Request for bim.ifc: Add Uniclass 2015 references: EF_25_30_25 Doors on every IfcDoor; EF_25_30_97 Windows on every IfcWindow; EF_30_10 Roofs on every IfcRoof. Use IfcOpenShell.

First a look at what the model holds.

```python
import ifcopenshell

model = ifcopenshell.open("bim.ifc")
print(model.schema)
print("classifications:", [c.Name for c in model.by_type("IfcClassification")])
for ifc_class in ("IfcDoor", "IfcRoof", "IfcStair", "IfcWall", "IfcWindow"):
    print(ifc_class, len(model.by_type(ifc_class)))
```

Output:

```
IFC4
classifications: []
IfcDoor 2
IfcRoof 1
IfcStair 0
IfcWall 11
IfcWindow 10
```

```python
import ifcopenshell
import ifcopenshell.api.classification

model = ifcopenshell.open("bim.ifc")

system = ifcopenshell.api.classification.add_classification(model, classification="Uniclass 2015")

codes = {
    "IfcDoor": ("EF_25_30_25", "Doors"),
    "IfcWindow": ("EF_25_30_97", "Windows"),
    "IfcRoof": ("EF_30_10", "Roofs"),
}
for ifc_class, (code, name) in codes.items():
    products = model.by_type(ifc_class)
    ifcopenshell.api.classification.add_reference(
        model, products=products, classification=system, identification=code, name=name
    )
    print(code, len(products))

model.write("bim_edited.ifc")
```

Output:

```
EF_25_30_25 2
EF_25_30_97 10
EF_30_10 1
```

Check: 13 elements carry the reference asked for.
